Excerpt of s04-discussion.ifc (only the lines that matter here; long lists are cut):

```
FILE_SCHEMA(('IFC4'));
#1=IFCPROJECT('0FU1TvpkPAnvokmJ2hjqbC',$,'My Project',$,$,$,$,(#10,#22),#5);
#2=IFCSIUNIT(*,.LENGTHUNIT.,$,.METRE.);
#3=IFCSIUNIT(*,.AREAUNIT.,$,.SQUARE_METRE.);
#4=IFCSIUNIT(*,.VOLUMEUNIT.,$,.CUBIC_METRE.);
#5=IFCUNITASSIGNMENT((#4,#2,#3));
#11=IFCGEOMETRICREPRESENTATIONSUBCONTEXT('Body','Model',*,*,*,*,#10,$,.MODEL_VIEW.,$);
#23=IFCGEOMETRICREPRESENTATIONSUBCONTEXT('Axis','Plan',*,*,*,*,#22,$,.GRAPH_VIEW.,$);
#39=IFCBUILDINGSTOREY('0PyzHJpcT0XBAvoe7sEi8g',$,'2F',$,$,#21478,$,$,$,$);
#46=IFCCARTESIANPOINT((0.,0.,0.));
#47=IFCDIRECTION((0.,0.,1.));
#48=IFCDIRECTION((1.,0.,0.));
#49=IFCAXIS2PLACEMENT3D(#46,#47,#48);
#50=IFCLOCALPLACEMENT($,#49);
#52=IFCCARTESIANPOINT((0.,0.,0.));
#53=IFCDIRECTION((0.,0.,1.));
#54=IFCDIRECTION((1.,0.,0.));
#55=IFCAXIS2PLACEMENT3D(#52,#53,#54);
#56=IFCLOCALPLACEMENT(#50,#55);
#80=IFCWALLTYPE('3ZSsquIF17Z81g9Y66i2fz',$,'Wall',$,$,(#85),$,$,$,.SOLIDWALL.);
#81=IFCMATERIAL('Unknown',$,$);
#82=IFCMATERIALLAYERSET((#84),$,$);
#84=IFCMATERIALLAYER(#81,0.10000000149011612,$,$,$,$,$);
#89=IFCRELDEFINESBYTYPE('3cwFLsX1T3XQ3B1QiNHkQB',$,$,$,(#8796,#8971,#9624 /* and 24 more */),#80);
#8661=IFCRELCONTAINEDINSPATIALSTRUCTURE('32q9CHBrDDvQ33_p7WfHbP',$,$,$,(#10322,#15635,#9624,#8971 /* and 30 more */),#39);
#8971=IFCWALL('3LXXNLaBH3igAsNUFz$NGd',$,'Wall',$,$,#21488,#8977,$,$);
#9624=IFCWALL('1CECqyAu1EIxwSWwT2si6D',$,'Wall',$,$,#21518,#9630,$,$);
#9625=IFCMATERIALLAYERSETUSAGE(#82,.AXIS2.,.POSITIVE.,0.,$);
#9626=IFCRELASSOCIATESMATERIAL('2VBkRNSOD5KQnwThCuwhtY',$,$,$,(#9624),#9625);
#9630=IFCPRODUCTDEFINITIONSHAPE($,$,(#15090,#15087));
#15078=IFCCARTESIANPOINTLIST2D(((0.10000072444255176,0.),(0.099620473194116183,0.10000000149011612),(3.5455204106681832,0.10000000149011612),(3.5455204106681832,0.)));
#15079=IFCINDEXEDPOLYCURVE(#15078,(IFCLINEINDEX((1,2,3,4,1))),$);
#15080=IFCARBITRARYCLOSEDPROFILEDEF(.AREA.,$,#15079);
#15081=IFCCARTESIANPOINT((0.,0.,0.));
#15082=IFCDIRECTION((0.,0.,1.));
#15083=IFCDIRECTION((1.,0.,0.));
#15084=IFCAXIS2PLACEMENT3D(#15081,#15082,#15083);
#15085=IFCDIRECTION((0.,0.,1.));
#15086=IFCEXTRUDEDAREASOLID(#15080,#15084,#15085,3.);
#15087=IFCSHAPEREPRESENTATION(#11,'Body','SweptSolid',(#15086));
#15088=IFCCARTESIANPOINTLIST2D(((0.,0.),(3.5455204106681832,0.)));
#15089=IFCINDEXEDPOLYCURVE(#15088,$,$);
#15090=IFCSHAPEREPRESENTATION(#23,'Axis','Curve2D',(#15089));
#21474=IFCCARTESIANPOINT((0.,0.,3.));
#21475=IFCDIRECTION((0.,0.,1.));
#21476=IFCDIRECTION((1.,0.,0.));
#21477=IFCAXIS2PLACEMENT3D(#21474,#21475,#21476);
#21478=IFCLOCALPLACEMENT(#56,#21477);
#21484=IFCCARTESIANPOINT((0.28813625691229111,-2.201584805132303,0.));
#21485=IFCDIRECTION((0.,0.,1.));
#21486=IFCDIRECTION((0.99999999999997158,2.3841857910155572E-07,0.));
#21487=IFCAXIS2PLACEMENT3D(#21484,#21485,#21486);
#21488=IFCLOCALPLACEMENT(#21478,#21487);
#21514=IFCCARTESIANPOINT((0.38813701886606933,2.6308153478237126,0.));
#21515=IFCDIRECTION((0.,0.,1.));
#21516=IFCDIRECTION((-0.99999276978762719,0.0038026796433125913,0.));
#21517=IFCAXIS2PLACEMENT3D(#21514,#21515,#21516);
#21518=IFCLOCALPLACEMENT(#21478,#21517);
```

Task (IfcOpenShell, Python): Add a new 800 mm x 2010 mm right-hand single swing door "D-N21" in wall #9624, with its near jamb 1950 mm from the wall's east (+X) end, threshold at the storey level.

```python
import numpy as np
import ifcopenshell
import ifcopenshell.api.feature
import ifcopenshell.api.geometry
import ifcopenshell.api.root
import ifcopenshell.api.spatial
import ifcopenshell.geom
import ifcopenshell.util.element
import ifcopenshell.util.placement
import ifcopenshell.util.representation
import ifcopenshell.util.shape
import ifcopenshell.util.unit

model = ifcopenshell.open("s04-discussion.ifc")
unit_scale = ifcopenshell.util.unit.calculate_unit_scale(model)
settings = ifcopenshell.geom.settings()


def volume(element):
    """Net volume in cubic metres, openings subtracted."""
    shape = ifcopenshell.geom.create_shape(settings, element)
    return ifcopenshell.util.shape.get_volume(shape.geometry)


wall = model.by_id(9624)
storey = ifcopenshell.util.element.get_container(wall, ifc_class="IfcBuildingStorey")
context = ifcopenshell.util.representation.get_context(model, "Model", "Body", "MODEL_VIEW")
before = volume(wall)

width, height, from_end, sill = 0.8, 2.01, 1.95, 0.0  # metres

# The wall runs along its own X axis, and the end named is its -X end.
wall_shape = ifcopenshell.geom.create_shape(settings, wall)
x, y, z = ifcopenshell.util.shape.get_vertices(wall_shape.geometry).T
start = x.min() + from_end
face, thickness = float(y.min()), float(y.max() - y.min())
wall_matrix = ifcopenshell.util.placement.get_local_placement(wall.ObjectPlacement)
level = ifcopenshell.util.placement.get_local_placement(storey.ObjectPlacement)[2, 3]


def in_wall(x, y):
    """Placement at x, y metres in the wall's axes, at sill height."""
    matrix = wall_matrix.copy()
    matrix[:, 3] = wall_matrix @ np.array([x / unit_scale, y / unit_scale, 0.0, 1.0])
    matrix[2, 3] = level + sill / unit_scale
    return matrix


# Opening: a box that overshoots both wall faces by 50 mm.
opening = ifcopenshell.api.root.create_entity(model, ifc_class="IfcOpeningElement", predefined_type="OPENING")
box = ifcopenshell.api.geometry.add_wall_representation(
    model, context=context, length=width, height=height, thickness=thickness + 0.1
)
ifcopenshell.api.geometry.assign_representation(model, product=opening, representation=box)
ifcopenshell.api.geometry.edit_object_placement(model, product=opening, matrix=in_wall(start, face - 0.05), is_si=False)
ifcopenshell.api.feature.add_feature(model, feature=opening, element=wall)

door = ifcopenshell.api.root.create_entity(model, ifc_class="IfcDoor", name="D-N21", predefined_type="DOOR")
door.OverallWidth, door.OverallHeight = width / unit_scale, height / unit_scale
door.OperationType = "SINGLE_SWING_RIGHT"
body = ifcopenshell.api.geometry.add_door_representation(
    model,
    context=context,
    overall_width=door.OverallWidth,
    overall_height=door.OverallHeight,
    operation_type="SINGLE_SWING_RIGHT",
    lining_properties={"LiningDepth": thickness / unit_scale, "ThresholdDepth": thickness / unit_scale},
)
ifcopenshell.api.geometry.assign_representation(model, product=door, representation=body)
ifcopenshell.api.spatial.assign_container(model, products=[door], relating_structure=storey)
ifcopenshell.api.feature.add_filling(model, opening=opening, element=door)

# The lining spans the wall, so the door starts at the wall face.
ifcopenshell.api.geometry.edit_object_placement(model, product=door, matrix=in_wall(start, face), is_si=False)

after = volume(wall)

print(f"wall volume {before:.3f} -> {after:.3f} m3")

model.write("s04-discussion_edited.ifc")
```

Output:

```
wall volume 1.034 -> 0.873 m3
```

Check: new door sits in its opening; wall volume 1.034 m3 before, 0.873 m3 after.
